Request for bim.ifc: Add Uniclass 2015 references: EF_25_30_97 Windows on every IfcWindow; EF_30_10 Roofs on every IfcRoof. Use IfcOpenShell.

First a look at what the model holds.

```python
import ifcopenshell

model = ifcopenshell.open("bim.ifc")
print(model.schema)
print("classifications:", [c.Name for c in model.by_type("IfcClassification")])
for ifc_class in ("IfcDoor", "IfcRoof", "IfcStair", "IfcWall", "IfcWindow"):
    print(ifc_class, len(model.by_type(ifc_class)))
```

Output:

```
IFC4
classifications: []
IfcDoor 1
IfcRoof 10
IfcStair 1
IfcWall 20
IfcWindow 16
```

```python
import ifcopenshell
import ifcopenshell.api.classification

model = ifcopenshell.open("bim.ifc")

system = ifcopenshell.api.classification.add_classification(model, classification="Uniclass 2015")

codes = {
    "IfcWindow": ("EF_25_30_97", "Windows"),
    "IfcRoof": ("EF_30_10", "Roofs"),
}
for ifc_class, (code, name) in codes.items():
    products = model.by_type(ifc_class)
    ifcopenshell.api.classification.add_reference(
        model, products=products, classification=system, identification=code, name=name
    )
    print(code, len(products))

model.write("bim_edited.ifc")
```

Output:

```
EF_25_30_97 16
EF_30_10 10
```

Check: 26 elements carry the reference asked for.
